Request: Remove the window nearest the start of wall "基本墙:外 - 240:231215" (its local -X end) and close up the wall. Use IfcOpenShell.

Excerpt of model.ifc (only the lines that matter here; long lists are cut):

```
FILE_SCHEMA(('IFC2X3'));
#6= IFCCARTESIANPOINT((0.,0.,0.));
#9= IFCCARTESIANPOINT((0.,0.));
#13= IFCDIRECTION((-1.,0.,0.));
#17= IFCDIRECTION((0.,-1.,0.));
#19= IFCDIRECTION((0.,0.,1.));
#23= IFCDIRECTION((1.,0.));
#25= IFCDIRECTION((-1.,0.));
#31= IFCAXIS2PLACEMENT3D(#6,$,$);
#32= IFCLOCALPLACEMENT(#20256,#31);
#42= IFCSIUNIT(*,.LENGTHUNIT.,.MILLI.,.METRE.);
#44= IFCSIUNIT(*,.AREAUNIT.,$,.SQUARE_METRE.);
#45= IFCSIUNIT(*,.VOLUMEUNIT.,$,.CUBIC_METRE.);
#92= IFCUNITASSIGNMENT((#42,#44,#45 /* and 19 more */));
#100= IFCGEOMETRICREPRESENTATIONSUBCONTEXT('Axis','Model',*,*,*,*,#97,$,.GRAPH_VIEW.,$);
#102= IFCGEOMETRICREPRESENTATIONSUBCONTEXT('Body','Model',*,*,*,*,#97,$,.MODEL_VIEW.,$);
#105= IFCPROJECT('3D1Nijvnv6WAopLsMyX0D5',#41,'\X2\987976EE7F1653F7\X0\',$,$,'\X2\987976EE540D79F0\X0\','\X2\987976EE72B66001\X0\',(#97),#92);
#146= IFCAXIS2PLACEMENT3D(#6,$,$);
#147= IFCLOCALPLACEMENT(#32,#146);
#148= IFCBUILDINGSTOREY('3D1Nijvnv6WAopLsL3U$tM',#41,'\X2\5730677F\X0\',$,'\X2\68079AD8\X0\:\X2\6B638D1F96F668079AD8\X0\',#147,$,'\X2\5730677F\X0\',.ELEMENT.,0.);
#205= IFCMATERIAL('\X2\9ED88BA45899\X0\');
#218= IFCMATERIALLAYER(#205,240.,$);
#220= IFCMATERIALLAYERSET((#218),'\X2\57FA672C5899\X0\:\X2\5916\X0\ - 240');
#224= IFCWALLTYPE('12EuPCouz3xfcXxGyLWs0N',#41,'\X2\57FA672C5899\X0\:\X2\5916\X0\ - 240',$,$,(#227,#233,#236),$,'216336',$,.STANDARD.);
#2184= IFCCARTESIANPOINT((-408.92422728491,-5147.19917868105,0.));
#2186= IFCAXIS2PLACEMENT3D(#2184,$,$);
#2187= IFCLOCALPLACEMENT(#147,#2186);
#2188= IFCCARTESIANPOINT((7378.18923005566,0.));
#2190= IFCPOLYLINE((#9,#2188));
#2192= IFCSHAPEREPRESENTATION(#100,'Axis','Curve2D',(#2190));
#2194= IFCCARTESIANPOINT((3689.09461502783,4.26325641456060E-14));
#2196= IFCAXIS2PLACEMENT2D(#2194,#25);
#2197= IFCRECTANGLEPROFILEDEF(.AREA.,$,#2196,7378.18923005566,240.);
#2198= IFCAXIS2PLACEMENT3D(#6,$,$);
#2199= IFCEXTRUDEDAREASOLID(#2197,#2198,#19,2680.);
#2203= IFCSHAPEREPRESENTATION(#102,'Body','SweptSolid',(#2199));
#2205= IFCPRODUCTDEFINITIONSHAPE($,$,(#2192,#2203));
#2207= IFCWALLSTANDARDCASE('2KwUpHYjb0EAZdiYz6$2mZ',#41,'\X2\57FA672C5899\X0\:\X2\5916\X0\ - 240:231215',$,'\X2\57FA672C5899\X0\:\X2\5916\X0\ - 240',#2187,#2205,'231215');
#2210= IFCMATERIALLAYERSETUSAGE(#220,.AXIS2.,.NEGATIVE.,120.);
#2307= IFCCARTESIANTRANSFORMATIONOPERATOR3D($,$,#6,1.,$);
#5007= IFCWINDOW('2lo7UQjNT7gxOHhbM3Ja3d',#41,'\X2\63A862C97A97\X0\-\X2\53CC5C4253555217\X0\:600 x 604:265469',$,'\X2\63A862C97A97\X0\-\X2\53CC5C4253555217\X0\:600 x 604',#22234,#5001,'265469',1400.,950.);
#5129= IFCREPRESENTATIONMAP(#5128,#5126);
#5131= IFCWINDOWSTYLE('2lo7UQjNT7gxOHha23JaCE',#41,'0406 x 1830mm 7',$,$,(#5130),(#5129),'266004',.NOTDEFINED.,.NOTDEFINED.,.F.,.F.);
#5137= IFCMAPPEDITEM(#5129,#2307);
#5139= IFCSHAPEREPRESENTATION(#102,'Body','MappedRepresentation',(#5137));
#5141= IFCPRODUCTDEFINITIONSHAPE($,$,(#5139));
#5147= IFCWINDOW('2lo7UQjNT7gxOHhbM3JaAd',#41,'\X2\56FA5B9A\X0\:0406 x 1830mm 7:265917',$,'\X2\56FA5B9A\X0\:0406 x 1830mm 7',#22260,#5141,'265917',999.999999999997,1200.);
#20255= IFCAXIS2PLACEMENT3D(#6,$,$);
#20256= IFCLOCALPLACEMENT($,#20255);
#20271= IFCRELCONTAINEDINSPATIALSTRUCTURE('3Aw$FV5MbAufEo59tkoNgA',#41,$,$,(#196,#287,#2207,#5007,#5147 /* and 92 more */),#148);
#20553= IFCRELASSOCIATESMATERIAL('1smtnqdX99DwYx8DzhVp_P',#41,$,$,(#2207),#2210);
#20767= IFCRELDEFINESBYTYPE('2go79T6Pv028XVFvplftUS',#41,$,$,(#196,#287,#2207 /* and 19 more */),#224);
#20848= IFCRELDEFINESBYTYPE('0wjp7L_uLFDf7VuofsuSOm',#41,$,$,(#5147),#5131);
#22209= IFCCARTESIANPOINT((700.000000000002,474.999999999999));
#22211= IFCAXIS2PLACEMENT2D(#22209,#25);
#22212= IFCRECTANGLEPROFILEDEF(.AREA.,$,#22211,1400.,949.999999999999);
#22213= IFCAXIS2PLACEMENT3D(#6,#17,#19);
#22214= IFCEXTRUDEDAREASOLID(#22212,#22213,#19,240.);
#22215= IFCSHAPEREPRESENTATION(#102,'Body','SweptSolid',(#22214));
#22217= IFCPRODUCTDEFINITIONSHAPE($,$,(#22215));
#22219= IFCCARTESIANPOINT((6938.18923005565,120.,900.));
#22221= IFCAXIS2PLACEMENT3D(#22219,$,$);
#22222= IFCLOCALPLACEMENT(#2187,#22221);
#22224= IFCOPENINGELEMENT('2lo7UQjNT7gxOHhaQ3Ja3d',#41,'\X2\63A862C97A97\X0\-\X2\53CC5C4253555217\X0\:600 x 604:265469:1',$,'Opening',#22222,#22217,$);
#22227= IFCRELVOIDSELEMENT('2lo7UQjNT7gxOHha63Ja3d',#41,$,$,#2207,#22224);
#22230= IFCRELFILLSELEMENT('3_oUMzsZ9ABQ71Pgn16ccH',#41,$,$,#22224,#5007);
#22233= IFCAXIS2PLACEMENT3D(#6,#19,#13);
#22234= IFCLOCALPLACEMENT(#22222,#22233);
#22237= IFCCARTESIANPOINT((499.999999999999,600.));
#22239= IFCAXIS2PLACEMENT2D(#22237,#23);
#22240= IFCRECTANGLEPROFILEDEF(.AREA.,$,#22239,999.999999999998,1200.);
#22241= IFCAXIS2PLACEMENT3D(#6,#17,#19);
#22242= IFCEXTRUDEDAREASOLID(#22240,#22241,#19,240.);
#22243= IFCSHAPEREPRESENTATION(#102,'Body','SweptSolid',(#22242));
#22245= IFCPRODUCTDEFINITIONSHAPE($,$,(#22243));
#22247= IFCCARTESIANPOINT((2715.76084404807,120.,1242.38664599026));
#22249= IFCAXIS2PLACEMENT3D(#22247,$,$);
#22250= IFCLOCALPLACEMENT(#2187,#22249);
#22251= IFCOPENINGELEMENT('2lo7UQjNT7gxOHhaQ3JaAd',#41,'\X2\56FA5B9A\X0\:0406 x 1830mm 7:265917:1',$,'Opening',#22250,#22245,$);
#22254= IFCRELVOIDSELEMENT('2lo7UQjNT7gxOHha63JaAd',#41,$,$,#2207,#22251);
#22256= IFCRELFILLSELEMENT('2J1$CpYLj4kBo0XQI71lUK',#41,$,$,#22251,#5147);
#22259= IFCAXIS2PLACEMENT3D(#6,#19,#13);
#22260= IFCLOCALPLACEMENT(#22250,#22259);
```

```python
import ifcopenshell
import ifcopenshell.api.feature
import ifcopenshell.api.root
import ifcopenshell.geom
import ifcopenshell.util.shape

model = ifcopenshell.open("model.ifc")
settings = ifcopenshell.geom.settings()


def volume(element):
    """Net volume in cubic metres, openings subtracted."""
    shape = ifcopenshell.geom.create_shape(settings, element)
    return ifcopenshell.util.shape.get_volume(shape.geometry)


window = model.by_id(5147)
opening = window.FillsVoids[0].RelatingOpeningElement
wall = opening.VoidsElements[0].RelatingBuildingElement
before = volume(wall)

ifcopenshell.api.root.remove_product(model, product=window)
ifcopenshell.api.feature.remove_feature(model, feature=opening)

after = volume(wall)

print(f"wall volume {before:.3f} -> {after:.3f} m3")

model.write("model_v2.ifc")
```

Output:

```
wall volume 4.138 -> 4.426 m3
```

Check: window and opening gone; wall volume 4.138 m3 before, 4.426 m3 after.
